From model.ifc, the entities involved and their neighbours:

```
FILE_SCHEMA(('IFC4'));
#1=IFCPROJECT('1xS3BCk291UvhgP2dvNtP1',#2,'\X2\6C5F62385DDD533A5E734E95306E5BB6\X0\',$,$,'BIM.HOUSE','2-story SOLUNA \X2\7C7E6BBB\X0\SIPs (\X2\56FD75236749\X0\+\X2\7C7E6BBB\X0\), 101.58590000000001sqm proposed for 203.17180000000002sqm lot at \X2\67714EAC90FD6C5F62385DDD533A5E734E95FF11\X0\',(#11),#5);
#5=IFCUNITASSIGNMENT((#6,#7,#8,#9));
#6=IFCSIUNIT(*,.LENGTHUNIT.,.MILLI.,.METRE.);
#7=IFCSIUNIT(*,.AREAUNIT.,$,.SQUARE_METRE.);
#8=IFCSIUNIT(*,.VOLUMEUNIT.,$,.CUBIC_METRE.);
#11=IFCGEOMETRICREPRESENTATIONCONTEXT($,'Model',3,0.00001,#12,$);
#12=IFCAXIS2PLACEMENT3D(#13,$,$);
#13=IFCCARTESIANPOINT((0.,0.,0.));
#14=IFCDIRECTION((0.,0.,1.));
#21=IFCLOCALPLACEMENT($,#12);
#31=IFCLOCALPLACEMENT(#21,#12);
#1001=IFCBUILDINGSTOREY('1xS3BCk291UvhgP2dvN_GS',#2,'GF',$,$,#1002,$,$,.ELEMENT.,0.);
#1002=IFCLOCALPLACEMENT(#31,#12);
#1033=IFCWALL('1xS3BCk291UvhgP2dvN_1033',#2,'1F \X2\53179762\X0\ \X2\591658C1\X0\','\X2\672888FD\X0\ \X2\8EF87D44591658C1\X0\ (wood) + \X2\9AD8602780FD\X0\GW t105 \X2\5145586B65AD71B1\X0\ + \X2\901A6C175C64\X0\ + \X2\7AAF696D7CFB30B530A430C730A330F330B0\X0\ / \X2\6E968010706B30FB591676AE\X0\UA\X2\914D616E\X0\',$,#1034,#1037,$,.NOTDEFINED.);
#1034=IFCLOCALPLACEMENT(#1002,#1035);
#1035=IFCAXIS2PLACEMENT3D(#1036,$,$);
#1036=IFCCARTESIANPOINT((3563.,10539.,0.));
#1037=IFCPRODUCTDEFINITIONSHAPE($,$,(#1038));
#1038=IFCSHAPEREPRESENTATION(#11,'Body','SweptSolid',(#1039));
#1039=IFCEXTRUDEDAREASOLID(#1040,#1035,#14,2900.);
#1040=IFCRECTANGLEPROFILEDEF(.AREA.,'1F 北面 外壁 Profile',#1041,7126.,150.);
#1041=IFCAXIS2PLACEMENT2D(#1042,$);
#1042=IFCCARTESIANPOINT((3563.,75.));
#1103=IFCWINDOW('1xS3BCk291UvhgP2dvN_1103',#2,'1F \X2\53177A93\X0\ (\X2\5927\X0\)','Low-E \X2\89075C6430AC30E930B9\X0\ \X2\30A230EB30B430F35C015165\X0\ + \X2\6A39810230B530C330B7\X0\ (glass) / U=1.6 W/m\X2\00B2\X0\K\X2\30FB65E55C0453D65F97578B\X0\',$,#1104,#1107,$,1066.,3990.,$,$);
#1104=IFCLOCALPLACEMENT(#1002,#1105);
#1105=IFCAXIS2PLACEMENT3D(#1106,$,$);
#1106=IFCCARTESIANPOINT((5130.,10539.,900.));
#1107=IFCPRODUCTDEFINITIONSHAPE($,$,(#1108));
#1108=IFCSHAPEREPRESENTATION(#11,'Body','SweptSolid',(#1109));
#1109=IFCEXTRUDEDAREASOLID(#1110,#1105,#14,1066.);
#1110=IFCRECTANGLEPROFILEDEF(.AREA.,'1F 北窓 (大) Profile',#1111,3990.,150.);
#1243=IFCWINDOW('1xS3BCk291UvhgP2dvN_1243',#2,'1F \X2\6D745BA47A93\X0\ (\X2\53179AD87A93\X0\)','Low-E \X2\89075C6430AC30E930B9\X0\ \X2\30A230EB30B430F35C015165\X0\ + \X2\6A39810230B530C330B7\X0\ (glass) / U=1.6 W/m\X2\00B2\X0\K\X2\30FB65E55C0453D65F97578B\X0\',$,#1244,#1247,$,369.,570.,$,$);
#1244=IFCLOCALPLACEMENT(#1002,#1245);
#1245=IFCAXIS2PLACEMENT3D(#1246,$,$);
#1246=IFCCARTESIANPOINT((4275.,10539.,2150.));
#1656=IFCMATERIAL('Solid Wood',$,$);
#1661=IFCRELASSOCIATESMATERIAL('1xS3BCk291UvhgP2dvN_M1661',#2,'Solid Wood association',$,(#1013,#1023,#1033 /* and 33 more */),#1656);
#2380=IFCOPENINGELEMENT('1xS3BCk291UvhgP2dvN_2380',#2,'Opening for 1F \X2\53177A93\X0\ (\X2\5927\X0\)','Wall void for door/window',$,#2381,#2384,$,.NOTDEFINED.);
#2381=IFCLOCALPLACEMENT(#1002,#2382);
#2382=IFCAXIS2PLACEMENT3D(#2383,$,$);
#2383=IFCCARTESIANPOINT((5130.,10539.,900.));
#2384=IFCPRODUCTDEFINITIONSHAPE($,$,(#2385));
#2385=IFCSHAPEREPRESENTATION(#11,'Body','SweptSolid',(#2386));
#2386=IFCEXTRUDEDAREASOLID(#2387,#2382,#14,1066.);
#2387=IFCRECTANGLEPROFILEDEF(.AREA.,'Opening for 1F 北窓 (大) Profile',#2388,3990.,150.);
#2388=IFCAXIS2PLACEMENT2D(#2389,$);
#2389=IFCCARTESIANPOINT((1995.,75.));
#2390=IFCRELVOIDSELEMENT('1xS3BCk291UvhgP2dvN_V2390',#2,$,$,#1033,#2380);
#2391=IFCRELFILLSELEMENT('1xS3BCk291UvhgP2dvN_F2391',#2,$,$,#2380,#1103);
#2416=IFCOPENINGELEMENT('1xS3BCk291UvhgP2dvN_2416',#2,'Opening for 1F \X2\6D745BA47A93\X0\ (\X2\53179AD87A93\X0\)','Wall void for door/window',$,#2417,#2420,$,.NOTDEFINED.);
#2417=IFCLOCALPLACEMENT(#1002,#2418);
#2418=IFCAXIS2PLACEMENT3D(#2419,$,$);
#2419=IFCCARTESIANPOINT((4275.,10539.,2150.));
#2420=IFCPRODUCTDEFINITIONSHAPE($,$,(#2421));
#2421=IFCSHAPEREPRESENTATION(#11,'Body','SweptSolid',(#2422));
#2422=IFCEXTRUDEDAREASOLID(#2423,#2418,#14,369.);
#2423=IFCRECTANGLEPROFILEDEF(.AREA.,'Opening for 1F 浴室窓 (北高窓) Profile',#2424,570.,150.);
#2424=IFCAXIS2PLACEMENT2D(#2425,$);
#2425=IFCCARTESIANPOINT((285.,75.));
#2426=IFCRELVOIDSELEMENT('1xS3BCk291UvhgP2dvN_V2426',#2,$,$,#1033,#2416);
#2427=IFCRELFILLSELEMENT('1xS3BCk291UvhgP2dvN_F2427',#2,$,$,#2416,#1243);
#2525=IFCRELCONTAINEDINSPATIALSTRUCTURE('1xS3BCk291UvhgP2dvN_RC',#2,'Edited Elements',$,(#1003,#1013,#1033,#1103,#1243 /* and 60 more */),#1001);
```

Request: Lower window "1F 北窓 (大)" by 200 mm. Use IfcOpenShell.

```python
import numpy as np
import ifcopenshell
import ifcopenshell.api.geometry
import ifcopenshell.util.placement
import ifcopenshell.util.unit

model = ifcopenshell.open("model.ifc")
unit_scale = ifcopenshell.util.unit.calculate_unit_scale(model)

window = model.by_guid("1xS3BCk291UvhgP2dvN_1103")
opening = window.FillsVoids[0].RelatingOpeningElement
dz = -0.2 / unit_scale

shift = np.array([0.0, 0.0, dz])
# The window is not placed relative to its opening, so move both.
for product in (opening, window):
    matrix = ifcopenshell.util.placement.get_local_placement(product.ObjectPlacement)
    matrix[:3, 3] += shift
    ifcopenshell.api.geometry.edit_object_placement(model, product=product, matrix=matrix, is_si=False)

print(f"moved by {dz * unit_scale:+.3f} m")

model.write("model_v2.ifc")
```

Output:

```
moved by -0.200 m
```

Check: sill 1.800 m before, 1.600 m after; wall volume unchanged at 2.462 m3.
